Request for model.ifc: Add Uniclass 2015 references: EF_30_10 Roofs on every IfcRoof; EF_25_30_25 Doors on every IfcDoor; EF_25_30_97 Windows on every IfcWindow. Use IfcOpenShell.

First a look at what the model holds.

```python
import ifcopenshell

model = ifcopenshell.open("model.ifc")
print(model.schema)
print("classifications:", [c.Name for c in model.by_type("IfcClassification")])
for ifc_class in ("IfcDoor", "IfcRoof", "IfcStair", "IfcWall", "IfcWindow"):
    print(ifc_class, len(model.by_type(ifc_class)))
```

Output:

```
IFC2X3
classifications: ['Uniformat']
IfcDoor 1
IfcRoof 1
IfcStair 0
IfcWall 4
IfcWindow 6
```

```python
import ifcopenshell
import ifcopenshell.api.classification

model = ifcopenshell.open("model.ifc")

# IFC2X3 requires Source and Edition and has no link from the project to the system.
system = model.create_entity("IfcClassification", Source="NBS", Edition="2015", Name="Uniclass 2015")

codes = {
    "IfcRoof": ("EF_30_10", "Roofs"),
    "IfcDoor": ("EF_25_30_25", "Doors"),
    "IfcWindow": ("EF_25_30_97", "Windows"),
}
for ifc_class, (code, name) in codes.items():
    products = model.by_type(ifc_class)
    ifcopenshell.api.classification.add_reference(
        model, products=products, classification=system, identification=code, name=name
    )
    print(code, len(products))

model.write("model-out.ifc")
```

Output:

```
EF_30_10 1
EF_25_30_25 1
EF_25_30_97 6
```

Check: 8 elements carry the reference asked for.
